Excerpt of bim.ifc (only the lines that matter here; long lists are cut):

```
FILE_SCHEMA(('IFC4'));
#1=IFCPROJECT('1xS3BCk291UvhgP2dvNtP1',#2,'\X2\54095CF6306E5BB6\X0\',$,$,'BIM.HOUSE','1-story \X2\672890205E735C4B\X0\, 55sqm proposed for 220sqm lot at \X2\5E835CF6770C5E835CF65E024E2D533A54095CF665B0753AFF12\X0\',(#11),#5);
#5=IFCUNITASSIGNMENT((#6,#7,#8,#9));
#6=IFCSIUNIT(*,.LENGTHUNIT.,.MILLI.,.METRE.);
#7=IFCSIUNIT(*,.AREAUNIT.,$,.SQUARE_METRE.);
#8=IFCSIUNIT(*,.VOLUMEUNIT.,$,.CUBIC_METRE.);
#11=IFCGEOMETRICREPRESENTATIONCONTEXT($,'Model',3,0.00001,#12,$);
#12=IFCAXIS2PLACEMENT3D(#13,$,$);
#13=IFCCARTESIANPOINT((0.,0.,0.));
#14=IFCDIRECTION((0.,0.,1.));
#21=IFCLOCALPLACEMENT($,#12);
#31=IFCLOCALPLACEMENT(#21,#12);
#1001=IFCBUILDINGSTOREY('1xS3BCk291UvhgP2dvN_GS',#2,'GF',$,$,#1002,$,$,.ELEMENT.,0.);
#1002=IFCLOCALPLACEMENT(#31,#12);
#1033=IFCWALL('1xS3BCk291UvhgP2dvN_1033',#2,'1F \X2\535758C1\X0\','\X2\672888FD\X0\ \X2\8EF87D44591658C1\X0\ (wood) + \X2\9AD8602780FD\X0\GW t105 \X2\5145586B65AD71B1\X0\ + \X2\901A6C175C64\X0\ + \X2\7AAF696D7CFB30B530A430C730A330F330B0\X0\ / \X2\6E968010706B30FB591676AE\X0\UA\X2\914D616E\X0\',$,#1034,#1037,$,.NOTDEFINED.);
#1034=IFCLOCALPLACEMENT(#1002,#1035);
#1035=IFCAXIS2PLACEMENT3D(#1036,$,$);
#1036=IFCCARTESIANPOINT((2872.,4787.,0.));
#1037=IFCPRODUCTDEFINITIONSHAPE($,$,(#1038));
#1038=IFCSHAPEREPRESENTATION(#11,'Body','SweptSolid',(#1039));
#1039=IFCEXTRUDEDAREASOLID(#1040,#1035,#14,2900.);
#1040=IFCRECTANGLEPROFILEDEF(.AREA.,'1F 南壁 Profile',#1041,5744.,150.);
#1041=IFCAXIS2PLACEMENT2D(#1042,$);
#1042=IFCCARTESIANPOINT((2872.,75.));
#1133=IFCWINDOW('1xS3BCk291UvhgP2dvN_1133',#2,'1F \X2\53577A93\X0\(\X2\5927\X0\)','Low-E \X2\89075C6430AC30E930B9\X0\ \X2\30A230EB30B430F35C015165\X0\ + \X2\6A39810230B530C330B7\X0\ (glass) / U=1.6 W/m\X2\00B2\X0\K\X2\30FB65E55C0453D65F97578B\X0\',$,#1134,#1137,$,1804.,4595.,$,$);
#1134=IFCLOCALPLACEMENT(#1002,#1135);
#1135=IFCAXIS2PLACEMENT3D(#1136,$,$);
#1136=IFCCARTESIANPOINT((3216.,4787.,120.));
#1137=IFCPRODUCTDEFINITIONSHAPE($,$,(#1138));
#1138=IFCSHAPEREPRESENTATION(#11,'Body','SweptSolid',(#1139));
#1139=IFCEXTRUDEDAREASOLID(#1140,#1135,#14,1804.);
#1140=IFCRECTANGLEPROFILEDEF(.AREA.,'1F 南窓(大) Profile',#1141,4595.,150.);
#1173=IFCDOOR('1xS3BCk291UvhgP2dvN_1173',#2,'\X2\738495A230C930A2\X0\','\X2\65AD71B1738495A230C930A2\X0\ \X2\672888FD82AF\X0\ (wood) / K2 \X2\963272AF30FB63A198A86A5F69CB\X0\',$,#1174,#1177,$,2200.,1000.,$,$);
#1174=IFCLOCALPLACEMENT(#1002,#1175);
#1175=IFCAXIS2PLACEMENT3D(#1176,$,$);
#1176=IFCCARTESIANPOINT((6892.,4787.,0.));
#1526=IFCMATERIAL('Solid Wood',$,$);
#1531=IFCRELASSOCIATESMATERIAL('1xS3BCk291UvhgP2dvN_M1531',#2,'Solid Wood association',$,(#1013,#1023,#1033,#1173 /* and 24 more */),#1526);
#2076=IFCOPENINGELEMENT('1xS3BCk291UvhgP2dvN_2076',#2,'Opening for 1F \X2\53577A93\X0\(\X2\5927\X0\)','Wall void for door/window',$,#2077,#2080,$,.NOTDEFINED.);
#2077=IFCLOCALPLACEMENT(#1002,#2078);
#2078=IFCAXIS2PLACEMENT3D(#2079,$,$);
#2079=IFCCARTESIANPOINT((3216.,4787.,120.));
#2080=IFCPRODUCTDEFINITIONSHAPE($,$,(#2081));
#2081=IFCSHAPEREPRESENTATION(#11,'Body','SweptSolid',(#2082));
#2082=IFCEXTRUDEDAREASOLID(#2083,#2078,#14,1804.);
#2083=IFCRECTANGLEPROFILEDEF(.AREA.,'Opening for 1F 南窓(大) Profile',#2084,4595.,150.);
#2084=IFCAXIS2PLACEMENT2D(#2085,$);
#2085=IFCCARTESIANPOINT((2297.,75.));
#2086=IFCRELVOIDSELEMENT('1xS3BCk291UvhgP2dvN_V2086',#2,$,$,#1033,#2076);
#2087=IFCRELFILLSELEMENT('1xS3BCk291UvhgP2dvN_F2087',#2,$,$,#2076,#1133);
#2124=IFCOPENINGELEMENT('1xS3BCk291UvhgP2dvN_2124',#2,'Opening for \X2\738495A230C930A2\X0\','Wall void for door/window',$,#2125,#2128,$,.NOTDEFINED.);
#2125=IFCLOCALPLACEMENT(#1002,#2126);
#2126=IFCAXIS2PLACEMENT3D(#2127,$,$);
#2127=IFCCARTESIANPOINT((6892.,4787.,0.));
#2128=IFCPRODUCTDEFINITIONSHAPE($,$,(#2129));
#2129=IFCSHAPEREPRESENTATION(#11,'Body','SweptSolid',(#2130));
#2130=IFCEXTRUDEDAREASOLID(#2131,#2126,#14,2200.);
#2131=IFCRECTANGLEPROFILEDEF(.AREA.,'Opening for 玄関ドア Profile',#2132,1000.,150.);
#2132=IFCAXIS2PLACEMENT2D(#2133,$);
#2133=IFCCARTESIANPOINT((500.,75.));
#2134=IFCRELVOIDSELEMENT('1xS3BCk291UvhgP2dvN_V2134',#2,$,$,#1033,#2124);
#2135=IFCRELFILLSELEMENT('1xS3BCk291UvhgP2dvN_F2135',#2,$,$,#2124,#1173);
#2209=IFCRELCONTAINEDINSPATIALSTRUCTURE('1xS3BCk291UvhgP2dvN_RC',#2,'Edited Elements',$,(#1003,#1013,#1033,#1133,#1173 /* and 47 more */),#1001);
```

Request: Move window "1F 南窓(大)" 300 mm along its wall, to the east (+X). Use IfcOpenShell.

```python
import ifcopenshell
import ifcopenshell.api.geometry
import ifcopenshell.util.placement
import ifcopenshell.util.unit

model = ifcopenshell.open("bim.ifc")
unit_scale = ifcopenshell.util.unit.calculate_unit_scale(model)

window = model.by_guid("1xS3BCk291UvhgP2dvN_1133")
opening = window.FillsVoids[0].RelatingOpeningElement
wall = opening.VoidsElements[0].RelatingBuildingElement

wall_matrix = ifcopenshell.util.placement.get_local_placement(wall.ObjectPlacement)
shift = wall_matrix[:3, 0] * 0.3 / unit_scale
before = ifcopenshell.util.placement.get_local_placement(window.ObjectPlacement)[:3, 3].copy()

# The window is not placed relative to its opening, so move both.
for product in (opening, window):
    matrix = ifcopenshell.util.placement.get_local_placement(product.ObjectPlacement)
    matrix[:3, 3] += shift
    ifcopenshell.api.geometry.edit_object_placement(model, product=product, matrix=matrix, is_si=False)

after = ifcopenshell.util.placement.get_local_placement(window.ObjectPlacement)[:3, 3]
print("window moved by", (after - before).round(3) + 0.0)

model.write("bim-out.ifc")
```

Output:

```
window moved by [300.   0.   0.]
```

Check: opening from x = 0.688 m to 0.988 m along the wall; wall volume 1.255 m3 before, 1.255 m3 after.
